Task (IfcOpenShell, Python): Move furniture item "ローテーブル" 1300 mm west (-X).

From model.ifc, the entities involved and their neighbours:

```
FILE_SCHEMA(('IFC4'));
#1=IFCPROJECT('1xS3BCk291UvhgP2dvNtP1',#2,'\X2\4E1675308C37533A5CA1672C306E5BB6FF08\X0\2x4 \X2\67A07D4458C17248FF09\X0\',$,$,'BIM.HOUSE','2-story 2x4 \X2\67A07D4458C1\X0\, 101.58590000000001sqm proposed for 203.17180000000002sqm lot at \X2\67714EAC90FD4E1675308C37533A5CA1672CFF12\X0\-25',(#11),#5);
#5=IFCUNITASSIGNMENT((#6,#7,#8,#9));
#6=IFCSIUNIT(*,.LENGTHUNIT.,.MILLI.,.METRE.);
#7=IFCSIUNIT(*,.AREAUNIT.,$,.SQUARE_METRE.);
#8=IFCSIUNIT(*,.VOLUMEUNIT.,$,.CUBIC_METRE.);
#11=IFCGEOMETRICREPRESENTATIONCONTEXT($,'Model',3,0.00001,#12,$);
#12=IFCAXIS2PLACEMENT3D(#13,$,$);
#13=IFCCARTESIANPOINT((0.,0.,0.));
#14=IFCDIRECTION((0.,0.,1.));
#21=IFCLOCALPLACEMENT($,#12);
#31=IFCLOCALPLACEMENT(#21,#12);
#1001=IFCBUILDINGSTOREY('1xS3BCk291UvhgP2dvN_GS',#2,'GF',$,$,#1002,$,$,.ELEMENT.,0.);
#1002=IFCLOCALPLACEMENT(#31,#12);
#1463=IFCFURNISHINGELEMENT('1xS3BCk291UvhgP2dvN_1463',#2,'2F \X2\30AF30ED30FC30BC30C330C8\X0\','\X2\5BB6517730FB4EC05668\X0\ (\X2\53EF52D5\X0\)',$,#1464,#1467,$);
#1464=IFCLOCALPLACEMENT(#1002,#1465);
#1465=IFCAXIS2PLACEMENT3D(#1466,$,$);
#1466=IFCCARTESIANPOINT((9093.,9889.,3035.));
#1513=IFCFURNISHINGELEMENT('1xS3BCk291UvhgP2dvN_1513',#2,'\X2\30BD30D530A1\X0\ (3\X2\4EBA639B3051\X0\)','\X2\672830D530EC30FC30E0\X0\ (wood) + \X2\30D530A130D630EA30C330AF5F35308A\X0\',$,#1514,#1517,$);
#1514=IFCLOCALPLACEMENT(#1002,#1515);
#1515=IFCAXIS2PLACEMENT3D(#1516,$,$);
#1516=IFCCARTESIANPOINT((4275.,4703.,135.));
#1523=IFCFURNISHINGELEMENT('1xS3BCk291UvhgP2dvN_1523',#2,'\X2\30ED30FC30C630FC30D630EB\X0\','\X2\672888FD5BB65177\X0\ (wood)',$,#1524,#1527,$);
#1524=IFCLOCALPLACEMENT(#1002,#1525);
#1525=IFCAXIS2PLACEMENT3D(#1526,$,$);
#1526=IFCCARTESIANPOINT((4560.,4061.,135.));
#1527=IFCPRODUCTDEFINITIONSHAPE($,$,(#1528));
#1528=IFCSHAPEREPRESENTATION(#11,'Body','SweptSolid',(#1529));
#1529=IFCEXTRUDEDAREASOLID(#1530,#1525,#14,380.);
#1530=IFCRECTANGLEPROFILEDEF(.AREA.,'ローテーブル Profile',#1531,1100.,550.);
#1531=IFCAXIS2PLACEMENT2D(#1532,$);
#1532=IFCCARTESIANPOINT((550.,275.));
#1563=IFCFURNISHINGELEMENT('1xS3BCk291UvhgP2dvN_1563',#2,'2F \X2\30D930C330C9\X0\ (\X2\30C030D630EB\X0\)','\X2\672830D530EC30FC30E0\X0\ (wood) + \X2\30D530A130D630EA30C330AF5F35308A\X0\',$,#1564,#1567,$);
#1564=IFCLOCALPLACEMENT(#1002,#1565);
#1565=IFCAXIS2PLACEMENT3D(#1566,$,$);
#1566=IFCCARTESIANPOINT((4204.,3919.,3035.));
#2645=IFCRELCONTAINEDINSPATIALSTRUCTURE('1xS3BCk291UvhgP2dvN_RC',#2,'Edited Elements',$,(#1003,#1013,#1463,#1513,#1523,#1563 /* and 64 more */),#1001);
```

```python
import ifcopenshell
import ifcopenshell.api.geometry
import ifcopenshell.util.placement
import ifcopenshell.util.unit

model = ifcopenshell.open("model.ifc")
unit_scale = ifcopenshell.util.unit.calculate_unit_scale(model)

item = model.by_guid("1xS3BCk291UvhgP2dvN_1523")
matrix = ifcopenshell.util.placement.get_local_placement(item.ObjectPlacement)
matrix[0, 3] -= 1.3 / unit_scale
ifcopenshell.api.geometry.edit_object_placement(model, product=item, matrix=matrix, is_si=False)

print(ifcopenshell.util.placement.get_local_placement(item.ObjectPlacement).round(3) + 0.0)

model.write("model_edited.ifc")
```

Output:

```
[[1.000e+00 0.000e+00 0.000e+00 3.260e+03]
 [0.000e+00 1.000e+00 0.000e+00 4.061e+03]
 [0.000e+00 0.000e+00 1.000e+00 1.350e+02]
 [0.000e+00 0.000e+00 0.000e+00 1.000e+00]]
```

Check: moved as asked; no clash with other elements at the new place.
